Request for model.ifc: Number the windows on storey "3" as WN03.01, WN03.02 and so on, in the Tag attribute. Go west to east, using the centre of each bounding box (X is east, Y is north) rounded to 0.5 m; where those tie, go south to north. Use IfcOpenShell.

First a look at what the model holds.

```python
import ifcopenshell
import ifcopenshell.util.element
import ifcopenshell.util.placement

model = ifcopenshell.open("model.ifc")
print(model.schema)
storey = next(s for s in model.by_type("IfcBuildingStorey") if s.Name == "3")
windows = [e for e in ifcopenshell.util.element.get_decomposition(storey) if e.is_a("IfcWindow")]
for e in sorted(windows, key=lambda e: e.id()):
    origin = ifcopenshell.util.placement.get_local_placement(e.ObjectPlacement)[:3, 3]
    print(e.id(), e.Tag, e.Name, origin.round(2) + 0.0, sep=" | ")
```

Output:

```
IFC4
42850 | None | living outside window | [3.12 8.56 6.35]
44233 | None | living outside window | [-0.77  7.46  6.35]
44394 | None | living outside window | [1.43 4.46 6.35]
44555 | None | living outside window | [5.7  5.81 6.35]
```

```python
import ifcopenshell
import ifcopenshell.geom
import ifcopenshell.util.element
import ifcopenshell.util.shape

model = ifcopenshell.open("model.ifc")
settings = ifcopenshell.geom.settings()
settings.set("use-world-coords", True)


def centre(element):
    shape = ifcopenshell.geom.create_shape(settings, element)
    return ifcopenshell.util.shape.get_bbox_centroid(shape.geometry)


storey = next(s for s in model.by_type("IfcBuildingStorey") if s.Name == "3")
windows = [e for e in ifcopenshell.util.element.get_decomposition(storey) if e.is_a("IfcWindow")]

# Insertion points can sit at a corner or the storey origin, so sort by the geometry (in metres).
centres = {e: centre(e) for e in windows}
windows.sort(key=lambda e: (round(centres[e][0] / 0.5), centres[e][1]))

for i, e in enumerate(windows, start=1):
    number = f"WN03.{i:02d}"
    e.Tag = number
    print(e.id(), number)

model.write("model_updated.ifc")
```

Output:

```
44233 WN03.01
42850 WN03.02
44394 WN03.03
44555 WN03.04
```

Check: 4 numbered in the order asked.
